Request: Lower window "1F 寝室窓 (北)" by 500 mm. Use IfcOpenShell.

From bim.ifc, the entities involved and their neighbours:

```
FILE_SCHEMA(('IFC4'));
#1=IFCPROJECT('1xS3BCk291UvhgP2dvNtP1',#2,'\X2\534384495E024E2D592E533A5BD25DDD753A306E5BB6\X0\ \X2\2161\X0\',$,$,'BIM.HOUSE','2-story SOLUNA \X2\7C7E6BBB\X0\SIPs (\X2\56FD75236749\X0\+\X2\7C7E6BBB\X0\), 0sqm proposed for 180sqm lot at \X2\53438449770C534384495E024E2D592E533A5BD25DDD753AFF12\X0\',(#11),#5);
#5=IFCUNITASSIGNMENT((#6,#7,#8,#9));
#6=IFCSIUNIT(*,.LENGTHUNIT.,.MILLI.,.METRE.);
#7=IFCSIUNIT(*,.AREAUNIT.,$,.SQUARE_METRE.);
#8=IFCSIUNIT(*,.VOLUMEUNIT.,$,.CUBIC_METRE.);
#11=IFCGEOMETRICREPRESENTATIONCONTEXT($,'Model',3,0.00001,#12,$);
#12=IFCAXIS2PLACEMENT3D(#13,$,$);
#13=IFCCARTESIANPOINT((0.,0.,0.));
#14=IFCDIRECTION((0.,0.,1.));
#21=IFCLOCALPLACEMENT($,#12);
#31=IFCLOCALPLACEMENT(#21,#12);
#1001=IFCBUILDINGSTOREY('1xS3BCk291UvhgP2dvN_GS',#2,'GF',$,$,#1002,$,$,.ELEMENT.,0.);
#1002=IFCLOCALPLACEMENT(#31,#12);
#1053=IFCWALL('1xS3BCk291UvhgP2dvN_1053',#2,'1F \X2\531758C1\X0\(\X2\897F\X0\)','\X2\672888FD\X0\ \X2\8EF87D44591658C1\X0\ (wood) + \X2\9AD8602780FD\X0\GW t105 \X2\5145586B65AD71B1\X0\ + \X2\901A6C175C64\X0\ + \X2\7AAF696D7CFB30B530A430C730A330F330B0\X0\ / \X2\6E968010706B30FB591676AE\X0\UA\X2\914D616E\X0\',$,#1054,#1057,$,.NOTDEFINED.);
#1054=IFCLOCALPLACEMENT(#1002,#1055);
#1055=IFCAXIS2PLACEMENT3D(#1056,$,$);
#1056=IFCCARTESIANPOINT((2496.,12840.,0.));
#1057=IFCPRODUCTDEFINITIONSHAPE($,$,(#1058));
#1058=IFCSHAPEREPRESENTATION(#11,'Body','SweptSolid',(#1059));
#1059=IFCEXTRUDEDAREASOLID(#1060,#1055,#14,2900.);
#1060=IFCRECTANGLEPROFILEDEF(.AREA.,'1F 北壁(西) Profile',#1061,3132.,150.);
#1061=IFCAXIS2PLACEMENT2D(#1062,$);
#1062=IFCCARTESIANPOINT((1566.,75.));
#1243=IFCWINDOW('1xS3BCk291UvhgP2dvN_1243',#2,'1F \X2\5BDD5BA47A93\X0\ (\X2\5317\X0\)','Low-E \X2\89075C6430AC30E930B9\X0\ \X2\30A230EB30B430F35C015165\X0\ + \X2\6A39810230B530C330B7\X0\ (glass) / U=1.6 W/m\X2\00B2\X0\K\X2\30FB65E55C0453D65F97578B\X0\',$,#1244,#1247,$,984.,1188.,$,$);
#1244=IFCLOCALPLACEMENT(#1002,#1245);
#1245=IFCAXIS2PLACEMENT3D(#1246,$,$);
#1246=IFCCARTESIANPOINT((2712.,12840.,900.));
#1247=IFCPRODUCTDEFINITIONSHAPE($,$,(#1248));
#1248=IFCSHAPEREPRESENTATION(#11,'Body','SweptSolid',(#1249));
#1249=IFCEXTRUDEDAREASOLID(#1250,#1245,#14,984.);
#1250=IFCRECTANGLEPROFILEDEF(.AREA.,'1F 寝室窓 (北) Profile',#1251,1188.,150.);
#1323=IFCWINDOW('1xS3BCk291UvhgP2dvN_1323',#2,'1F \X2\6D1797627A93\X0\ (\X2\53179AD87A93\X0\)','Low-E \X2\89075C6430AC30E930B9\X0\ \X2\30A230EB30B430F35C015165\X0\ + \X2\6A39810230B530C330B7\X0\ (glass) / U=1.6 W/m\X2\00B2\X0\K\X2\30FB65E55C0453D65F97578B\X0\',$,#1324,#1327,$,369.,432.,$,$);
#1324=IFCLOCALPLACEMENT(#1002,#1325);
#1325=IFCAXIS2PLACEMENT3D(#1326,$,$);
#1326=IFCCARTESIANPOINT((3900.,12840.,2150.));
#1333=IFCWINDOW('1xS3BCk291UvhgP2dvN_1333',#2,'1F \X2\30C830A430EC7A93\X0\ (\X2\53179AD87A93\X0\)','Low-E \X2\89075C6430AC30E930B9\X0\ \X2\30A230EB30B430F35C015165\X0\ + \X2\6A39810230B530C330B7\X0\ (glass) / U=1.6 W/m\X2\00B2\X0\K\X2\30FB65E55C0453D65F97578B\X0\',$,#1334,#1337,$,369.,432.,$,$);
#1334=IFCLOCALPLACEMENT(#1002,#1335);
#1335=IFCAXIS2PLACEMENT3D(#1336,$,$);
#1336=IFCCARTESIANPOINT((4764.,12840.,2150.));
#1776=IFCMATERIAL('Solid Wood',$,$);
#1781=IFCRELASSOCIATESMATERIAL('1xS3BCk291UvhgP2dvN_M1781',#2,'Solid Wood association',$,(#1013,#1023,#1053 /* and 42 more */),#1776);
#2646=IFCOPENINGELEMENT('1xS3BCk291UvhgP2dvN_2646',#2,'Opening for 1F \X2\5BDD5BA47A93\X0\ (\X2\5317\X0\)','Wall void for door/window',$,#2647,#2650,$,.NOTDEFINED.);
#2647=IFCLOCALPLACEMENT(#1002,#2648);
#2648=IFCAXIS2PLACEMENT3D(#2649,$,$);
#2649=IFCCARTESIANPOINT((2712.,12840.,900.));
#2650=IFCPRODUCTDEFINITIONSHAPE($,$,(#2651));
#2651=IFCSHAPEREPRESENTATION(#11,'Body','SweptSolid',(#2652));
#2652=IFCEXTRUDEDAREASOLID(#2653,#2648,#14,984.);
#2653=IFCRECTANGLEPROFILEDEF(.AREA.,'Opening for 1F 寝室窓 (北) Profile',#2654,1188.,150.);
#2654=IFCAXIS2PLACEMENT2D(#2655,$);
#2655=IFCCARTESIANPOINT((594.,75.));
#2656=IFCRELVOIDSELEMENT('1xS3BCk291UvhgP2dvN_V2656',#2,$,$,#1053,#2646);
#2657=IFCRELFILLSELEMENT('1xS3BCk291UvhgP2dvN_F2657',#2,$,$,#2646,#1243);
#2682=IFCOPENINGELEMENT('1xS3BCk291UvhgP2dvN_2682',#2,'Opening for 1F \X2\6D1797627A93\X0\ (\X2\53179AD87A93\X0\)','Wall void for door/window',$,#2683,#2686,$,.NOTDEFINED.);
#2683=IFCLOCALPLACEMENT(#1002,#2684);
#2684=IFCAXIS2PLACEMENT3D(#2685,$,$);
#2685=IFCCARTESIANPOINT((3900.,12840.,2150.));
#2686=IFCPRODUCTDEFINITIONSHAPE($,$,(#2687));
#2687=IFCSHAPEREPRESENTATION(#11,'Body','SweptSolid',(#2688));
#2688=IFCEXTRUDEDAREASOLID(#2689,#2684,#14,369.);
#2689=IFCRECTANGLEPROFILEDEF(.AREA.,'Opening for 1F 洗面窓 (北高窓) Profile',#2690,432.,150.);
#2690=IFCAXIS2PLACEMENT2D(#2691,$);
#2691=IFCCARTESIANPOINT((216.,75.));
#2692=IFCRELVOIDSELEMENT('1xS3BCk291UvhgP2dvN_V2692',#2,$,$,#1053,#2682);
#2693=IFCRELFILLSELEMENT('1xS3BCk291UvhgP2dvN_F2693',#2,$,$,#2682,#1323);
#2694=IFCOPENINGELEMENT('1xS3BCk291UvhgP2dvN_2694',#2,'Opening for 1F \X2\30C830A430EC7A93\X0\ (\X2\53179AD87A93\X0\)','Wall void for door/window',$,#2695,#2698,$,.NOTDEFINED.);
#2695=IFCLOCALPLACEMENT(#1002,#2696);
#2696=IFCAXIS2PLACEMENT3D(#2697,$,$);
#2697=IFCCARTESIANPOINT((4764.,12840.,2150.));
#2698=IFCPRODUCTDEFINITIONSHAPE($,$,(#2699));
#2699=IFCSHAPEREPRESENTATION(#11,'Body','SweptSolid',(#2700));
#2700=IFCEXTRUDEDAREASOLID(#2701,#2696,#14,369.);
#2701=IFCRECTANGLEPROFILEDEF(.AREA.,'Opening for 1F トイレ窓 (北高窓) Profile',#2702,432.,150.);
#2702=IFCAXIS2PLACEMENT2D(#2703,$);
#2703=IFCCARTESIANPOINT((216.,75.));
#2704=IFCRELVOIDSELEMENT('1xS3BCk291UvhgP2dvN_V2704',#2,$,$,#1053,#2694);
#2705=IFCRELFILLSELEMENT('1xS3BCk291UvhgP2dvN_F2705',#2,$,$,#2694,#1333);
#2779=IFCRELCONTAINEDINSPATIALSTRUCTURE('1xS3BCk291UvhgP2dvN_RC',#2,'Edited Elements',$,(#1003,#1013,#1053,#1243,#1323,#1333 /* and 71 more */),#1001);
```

```python
import numpy as np
import ifcopenshell
import ifcopenshell.api.geometry
import ifcopenshell.util.placement
import ifcopenshell.util.unit

model = ifcopenshell.open("bim.ifc")
unit_scale = ifcopenshell.util.unit.calculate_unit_scale(model)

window = model.by_guid("1xS3BCk291UvhgP2dvN_1243")
opening = window.FillsVoids[0].RelatingOpeningElement
dz = -0.5 / unit_scale

shift = np.array([0.0, 0.0, dz])
# The window is not placed relative to its opening, so move both.
for product in (opening, window):
    matrix = ifcopenshell.util.placement.get_local_placement(product.ObjectPlacement)
    matrix[:3, 3] += shift
    ifcopenshell.api.geometry.edit_object_placement(model, product=product, matrix=matrix, is_si=False)

print(f"moved by {dz * unit_scale:+.3f} m")

model.write("bim_updated.ifc")
```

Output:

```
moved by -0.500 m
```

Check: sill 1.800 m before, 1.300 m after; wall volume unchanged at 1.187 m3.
